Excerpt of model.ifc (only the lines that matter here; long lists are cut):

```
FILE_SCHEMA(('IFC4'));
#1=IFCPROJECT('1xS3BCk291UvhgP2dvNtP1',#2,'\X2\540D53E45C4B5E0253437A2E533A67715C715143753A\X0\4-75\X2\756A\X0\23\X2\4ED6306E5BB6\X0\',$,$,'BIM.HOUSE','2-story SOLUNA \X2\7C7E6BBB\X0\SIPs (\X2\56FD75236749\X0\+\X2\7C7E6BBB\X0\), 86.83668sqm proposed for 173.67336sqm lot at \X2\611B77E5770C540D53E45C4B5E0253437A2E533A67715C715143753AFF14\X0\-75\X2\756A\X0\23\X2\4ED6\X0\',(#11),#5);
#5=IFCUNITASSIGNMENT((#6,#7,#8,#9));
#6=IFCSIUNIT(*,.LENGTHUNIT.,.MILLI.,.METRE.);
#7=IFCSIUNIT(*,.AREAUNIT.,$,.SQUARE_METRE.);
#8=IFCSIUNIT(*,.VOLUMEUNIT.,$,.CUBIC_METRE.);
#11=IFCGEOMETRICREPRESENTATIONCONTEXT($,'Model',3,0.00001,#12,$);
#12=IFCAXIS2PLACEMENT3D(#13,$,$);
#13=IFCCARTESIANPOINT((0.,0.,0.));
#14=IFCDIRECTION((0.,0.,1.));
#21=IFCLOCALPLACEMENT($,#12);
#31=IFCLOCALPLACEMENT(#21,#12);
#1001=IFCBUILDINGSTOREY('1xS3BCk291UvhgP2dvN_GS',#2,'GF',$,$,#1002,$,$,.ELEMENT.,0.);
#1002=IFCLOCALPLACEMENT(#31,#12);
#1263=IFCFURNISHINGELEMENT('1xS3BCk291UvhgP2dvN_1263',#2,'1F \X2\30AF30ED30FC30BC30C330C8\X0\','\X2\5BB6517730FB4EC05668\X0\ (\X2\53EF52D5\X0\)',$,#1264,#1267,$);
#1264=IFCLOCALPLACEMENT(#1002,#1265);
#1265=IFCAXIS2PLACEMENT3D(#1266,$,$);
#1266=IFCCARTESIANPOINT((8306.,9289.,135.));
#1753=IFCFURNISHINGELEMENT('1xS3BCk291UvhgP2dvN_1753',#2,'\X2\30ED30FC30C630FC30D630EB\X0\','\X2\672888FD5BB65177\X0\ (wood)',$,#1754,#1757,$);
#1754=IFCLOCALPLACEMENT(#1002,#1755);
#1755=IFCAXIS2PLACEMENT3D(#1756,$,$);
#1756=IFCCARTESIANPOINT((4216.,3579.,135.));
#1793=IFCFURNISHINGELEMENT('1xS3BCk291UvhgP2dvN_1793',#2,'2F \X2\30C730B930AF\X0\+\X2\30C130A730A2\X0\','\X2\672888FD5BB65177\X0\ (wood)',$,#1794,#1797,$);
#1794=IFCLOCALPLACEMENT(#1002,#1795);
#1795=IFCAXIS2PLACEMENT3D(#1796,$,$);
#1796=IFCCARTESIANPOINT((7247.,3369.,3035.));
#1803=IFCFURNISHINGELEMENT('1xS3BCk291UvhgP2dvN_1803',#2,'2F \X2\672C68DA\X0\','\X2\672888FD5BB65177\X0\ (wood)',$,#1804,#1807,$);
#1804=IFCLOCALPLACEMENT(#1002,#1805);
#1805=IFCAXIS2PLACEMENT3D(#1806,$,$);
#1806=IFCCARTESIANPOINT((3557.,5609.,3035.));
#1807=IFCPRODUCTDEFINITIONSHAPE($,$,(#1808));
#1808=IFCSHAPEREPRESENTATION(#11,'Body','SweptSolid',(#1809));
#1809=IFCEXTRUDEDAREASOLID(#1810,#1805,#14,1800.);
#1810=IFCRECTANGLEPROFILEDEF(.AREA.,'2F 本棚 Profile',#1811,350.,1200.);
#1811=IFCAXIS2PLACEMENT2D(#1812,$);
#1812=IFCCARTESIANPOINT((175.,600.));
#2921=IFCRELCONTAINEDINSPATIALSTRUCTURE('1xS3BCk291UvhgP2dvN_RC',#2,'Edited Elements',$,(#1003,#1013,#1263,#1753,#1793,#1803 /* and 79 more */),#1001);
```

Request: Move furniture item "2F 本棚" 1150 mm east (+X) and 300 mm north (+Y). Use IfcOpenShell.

```python
import ifcopenshell
import ifcopenshell.api.geometry
import ifcopenshell.util.placement

model = ifcopenshell.open("model.ifc")

item = model.by_guid("1xS3BCk291UvhgP2dvN_1803")
matrix = ifcopenshell.util.placement.get_local_placement(item.ObjectPlacement)
matrix[0, 3] += 1150.0
matrix[1, 3] += 300.0
ifcopenshell.api.geometry.edit_object_placement(model, product=item, matrix=matrix, is_si=False)

print(ifcopenshell.util.placement.get_local_placement(item.ObjectPlacement).round(3) + 0.0)

model.write("model_v2.ifc")
```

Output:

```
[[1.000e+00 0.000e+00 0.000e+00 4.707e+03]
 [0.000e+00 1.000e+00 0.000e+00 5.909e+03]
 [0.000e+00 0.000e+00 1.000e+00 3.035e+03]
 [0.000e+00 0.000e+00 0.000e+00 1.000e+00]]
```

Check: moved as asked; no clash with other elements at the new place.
